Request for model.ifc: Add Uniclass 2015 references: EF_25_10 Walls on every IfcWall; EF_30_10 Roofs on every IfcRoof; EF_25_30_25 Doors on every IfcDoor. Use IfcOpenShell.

First a look at what the model holds.

```python
import ifcopenshell

model = ifcopenshell.open("model.ifc")
print(model.schema)
print("classifications:", [c.Name for c in model.by_type("IfcClassification")])
for ifc_class in ("IfcDoor", "IfcRoof", "IfcStair", "IfcWall", "IfcWindow"):
    print(ifc_class, len(model.by_type(ifc_class)))
```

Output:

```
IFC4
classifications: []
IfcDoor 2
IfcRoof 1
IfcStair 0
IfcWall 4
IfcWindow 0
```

```python
import ifcopenshell
import ifcopenshell.api.classification

model = ifcopenshell.open("model.ifc")

system = ifcopenshell.api.classification.add_classification(model, classification="Uniclass 2015")

codes = {
    "IfcWall": ("EF_25_10", "Walls"),
    "IfcRoof": ("EF_30_10", "Roofs"),
    "IfcDoor": ("EF_25_30_25", "Doors"),
}
for ifc_class, (code, name) in codes.items():
    products = model.by_type(ifc_class)
    ifcopenshell.api.classification.add_reference(
        model, products=products, classification=system, identification=code, name=name
    )
    print(code, len(products))

model.write("model_rev.ifc")
```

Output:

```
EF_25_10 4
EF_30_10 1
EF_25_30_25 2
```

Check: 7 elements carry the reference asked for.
